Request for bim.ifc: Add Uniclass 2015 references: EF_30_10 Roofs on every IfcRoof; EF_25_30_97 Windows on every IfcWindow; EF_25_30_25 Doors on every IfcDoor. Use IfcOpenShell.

First a look at what the model holds.

```python
import ifcopenshell

model = ifcopenshell.open("bim.ifc")
print(model.schema)
print("classifications:", [c.Name for c in model.by_type("IfcClassification")])
for ifc_class in ("IfcDoor", "IfcRoof", "IfcStair", "IfcWall", "IfcWindow"):
    print(ifc_class, len(model.by_type(ifc_class)))
```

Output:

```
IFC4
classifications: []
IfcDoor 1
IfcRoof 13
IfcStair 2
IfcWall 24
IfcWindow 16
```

```python
import ifcopenshell
import ifcopenshell.api.classification

model = ifcopenshell.open("bim.ifc")

system = ifcopenshell.api.classification.add_classification(model, classification="Uniclass 2015")

codes = {
    "IfcRoof": ("EF_30_10", "Roofs"),
    "IfcWindow": ("EF_25_30_97", "Windows"),
    "IfcDoor": ("EF_25_30_25", "Doors"),
}
for ifc_class, (code, name) in codes.items():
    products = model.by_type(ifc_class)
    ifcopenshell.api.classification.add_reference(
        model, products=products, classification=system, identification=code, name=name
    )
    print(code, len(products))

model.write("bim_v2.ifc")
```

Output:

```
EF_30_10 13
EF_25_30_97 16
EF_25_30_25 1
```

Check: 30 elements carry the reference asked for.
